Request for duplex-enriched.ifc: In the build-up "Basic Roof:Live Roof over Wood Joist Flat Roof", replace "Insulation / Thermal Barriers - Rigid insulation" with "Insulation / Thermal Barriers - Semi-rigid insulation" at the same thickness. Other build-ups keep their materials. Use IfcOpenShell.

First a look at what the model holds.

```python
import ifcopenshell
import ifcopenshell.util.element

model = ifcopenshell.open("duplex-enriched.ifc")
print(model.schema)
for layer_set in model.by_type("IfcMaterialLayerSet"):
    if layer_set.LayerSetName == "Basic Roof:Live Roof over Wood Joist Flat Roof":
        for layer in layer_set.MaterialLayers:
            print(layer.id(), layer.Material and layer.Material.Name, layer.LayerThickness, sep=" | ")
        print(len(ifcopenshell.util.element.get_elements_by_material(model, layer_set)), "elements and types use it")
print(sorted(m.Name for m in model.by_type("IfcMaterial") if m.Name)[:60])
```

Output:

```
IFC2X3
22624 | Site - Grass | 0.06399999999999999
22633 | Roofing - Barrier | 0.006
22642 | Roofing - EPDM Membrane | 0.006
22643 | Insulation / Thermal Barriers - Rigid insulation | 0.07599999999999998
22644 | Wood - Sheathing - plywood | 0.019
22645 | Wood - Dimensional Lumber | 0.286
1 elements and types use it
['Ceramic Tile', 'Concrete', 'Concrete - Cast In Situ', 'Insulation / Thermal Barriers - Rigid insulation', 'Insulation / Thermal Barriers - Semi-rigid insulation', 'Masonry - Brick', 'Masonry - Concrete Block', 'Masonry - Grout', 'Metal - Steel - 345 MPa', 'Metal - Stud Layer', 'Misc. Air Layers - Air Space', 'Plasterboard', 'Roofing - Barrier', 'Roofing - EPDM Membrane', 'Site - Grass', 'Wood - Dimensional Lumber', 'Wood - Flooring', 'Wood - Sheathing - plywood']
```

```python
import ifcopenshell
import ifcopenshell.api.material

model = ifcopenshell.open("duplex-enriched.ifc")

layer_set = next(s for s in model.by_type("IfcMaterialLayerSet") if s.LayerSetName == "Basic Roof:Live Roof over Wood Joist Flat Roof")
layer = next(l for l in layer_set.MaterialLayers if l.Material and l.Material.Name == "Insulation / Thermal Barriers - Rigid insulation")
material = next(m for m in model.by_type("IfcMaterial") if m.Name == "Insulation / Thermal Barriers - Semi-rigid insulation")

# Point this one layer at the other material; renaming the old one would change it everywhere.
ifcopenshell.api.material.edit_layer(model, layer=layer, attributes={}, material=material)

print([l.Material.Name if l.Material else None for l in layer_set.MaterialLayers])

model.write("duplex-enriched_edited.ifc")
```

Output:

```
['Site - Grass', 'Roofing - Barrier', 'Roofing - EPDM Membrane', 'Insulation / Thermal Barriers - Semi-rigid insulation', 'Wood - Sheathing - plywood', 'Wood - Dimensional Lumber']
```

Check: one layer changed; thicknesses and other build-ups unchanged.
